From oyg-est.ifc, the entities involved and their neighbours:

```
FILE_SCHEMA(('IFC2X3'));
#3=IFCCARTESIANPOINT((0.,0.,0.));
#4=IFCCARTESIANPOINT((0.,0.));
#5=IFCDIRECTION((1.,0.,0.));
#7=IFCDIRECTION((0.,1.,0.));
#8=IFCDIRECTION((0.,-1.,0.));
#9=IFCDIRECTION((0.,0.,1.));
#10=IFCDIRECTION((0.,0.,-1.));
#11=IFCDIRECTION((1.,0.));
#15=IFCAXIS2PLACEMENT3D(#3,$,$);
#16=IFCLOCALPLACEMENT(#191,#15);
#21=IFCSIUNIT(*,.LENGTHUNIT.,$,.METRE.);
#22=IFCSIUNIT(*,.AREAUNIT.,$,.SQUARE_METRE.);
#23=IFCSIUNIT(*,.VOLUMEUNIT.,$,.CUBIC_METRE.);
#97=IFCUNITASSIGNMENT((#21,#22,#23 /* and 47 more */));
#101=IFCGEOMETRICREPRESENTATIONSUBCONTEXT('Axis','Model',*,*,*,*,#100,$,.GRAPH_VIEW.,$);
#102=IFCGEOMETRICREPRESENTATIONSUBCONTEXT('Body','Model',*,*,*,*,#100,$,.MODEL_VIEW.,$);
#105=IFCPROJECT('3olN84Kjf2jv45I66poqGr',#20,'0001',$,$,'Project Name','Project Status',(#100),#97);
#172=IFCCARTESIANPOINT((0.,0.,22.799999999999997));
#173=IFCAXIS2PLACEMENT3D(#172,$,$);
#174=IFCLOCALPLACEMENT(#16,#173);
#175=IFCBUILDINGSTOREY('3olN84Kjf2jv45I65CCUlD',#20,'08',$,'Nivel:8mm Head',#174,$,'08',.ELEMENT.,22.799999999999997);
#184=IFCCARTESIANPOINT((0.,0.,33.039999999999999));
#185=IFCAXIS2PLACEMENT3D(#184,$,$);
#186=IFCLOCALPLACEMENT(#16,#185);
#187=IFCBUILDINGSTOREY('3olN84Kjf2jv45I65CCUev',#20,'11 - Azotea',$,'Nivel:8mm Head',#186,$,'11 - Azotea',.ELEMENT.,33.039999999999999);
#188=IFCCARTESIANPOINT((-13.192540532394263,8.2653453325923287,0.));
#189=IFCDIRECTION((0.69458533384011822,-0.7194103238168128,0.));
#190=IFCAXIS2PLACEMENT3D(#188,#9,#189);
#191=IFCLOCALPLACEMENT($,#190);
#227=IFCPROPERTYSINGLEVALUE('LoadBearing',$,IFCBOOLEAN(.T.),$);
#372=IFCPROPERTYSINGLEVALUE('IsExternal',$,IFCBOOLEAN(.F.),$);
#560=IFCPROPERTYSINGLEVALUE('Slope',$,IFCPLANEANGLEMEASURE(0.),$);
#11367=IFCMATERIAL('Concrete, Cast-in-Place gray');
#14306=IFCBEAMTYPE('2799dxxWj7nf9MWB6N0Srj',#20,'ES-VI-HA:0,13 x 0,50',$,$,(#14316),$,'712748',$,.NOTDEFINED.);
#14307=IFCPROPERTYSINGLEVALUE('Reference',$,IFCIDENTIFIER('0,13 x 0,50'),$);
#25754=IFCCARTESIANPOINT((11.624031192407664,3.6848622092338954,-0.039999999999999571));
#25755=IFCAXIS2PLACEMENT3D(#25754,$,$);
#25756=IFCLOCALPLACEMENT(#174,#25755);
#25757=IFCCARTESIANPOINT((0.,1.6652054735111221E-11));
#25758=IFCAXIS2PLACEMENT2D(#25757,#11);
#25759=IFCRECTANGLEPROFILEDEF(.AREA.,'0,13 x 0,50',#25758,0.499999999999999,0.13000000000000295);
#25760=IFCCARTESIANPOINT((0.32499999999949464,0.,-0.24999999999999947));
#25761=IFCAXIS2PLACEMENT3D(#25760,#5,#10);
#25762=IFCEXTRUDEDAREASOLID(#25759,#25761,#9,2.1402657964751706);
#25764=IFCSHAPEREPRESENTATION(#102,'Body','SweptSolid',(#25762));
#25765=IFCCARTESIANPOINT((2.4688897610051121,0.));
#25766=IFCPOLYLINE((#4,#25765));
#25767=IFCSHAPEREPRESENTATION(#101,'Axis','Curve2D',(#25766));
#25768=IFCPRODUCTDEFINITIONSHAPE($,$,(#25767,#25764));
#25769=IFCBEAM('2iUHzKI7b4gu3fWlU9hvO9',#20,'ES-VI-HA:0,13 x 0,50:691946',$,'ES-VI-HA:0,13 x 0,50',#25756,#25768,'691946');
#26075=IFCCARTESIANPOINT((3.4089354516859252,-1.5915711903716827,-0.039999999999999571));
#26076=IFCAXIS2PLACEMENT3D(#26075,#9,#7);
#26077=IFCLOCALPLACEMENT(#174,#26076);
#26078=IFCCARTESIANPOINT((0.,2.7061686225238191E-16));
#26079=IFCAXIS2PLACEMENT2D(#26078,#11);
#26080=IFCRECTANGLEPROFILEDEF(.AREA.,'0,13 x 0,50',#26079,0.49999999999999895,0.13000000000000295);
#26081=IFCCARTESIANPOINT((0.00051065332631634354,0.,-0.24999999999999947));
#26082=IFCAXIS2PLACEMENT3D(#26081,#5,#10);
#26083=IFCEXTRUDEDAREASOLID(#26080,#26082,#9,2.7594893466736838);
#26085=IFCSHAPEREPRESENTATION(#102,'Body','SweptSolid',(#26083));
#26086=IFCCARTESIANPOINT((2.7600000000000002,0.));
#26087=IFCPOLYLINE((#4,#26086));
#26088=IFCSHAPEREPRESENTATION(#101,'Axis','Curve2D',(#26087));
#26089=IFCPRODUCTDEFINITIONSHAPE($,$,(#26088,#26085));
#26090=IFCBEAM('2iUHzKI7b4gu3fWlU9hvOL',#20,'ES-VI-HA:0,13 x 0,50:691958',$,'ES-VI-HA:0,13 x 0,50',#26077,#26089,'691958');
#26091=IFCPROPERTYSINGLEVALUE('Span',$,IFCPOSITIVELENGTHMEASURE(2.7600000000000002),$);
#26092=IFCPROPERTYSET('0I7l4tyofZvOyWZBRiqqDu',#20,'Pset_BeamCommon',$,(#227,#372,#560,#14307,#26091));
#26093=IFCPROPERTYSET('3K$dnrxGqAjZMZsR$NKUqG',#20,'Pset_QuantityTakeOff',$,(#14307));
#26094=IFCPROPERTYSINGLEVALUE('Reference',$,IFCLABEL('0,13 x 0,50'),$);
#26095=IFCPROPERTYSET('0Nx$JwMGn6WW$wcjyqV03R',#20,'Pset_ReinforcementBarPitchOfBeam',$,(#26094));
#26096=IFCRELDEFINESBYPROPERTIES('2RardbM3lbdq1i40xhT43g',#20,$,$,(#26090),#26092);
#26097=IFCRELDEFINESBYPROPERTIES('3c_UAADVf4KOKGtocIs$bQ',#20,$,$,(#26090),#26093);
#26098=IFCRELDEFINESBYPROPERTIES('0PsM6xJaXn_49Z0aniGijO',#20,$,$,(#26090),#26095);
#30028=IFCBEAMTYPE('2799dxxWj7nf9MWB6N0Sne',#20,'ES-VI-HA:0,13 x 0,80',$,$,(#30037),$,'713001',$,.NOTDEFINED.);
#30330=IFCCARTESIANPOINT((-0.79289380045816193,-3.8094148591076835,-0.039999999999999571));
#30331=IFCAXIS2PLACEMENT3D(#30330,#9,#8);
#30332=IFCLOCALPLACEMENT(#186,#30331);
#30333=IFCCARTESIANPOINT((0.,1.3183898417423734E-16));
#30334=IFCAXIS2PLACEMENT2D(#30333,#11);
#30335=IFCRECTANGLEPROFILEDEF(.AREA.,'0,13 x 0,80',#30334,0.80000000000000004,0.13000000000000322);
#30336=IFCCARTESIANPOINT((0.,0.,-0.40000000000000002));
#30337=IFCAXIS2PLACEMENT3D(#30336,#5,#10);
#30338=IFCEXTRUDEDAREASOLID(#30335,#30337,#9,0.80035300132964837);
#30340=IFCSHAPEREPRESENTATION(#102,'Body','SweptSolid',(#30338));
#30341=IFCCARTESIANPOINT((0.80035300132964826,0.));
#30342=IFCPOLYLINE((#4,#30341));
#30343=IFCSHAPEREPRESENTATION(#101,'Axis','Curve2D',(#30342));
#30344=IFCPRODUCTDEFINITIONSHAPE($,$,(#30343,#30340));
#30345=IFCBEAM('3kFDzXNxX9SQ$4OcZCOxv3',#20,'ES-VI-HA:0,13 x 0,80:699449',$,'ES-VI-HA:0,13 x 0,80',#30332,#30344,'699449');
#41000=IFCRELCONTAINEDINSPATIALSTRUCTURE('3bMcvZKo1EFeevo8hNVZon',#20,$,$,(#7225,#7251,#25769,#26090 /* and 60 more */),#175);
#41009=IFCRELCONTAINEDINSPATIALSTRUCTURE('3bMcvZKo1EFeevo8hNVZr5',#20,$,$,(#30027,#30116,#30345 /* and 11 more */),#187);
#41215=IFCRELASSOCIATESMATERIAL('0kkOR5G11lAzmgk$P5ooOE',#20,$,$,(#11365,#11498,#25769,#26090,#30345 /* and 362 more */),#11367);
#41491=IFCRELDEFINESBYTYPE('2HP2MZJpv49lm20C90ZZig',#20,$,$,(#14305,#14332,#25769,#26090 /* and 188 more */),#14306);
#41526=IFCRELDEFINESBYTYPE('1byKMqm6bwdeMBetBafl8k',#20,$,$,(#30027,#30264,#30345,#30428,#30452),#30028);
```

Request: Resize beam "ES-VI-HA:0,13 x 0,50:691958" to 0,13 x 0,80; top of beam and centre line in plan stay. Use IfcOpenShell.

```python
import ifcopenshell
import ifcopenshell.api.pset
import ifcopenshell.api.type
import ifcopenshell.util.element
import ifcopenshell.util.representation

model = ifcopenshell.open("oyg-est.ifc")

member = model.by_guid("2iUHzKI7b4gu3fWlU9hvOL")
source = next(p for p in model.by_type("IfcRectangleProfileDef") if p.ProfileName == "0,13 x 0,80")

body = ifcopenshell.util.representation.get_representation(member, "Model", "Body")
solid = body.Items[0]
old_profile = solid.SweptArea

# Copy the section's sizes but keep this member's own profile position.
profile = ifcopenshell.util.element.copy(model, source)
# Profiles are centred, so shift by half the change in depth to hold the top.
shift = (old_profile.XDim - profile.XDim) / 2
x, y = old_profile.Position.Location.Coordinates
up = (-1.0, 0.0)  # upwards, in the solid's own plane
location = model.createIfcCartesianPoint((x + up[0] * shift, y + up[1] * shift))
profile.Position = model.createIfcAxis2Placement2D(location, old_profile.Position.RefDirection)
solid.SweptArea = profile
if not model.get_total_inverses(old_profile):
    ifcopenshell.util.element.remove_deep2(model, old_profile)

new_type = model.by_guid("2799dxxWj7nf9MWB6N0Sne")
ifcopenshell.api.type.assign_type(
    model, related_objects=[member], relating_type=new_type, should_map_representations=False
)
member.Name = member.Name.replace("0,13 x 0,50", "0,13 x 0,80")
member.ObjectType = "ES-VI-HA:0,13 x 0,80"
pset = model.by_id(ifcopenshell.util.element.get_pset(member, "Pset_BeamCommon", should_inherit=False)["id"])
ifcopenshell.api.pset.edit_pset(model, pset=pset, properties={"Reference": "0,13 x 0,80"})
pset = model.by_id(ifcopenshell.util.element.get_pset(member, "Pset_QuantityTakeOff", should_inherit=False)["id"])
ifcopenshell.api.pset.edit_pset(model, pset=pset, properties={"Reference": "0,13 x 0,80"})
pset = model.by_id(ifcopenshell.util.element.get_pset(member, "Pset_ReinforcementBarPitchOfBeam", should_inherit=False)["id"])
ifcopenshell.api.pset.edit_pset(model, pset=pset, properties={"Reference": "0,13 x 0,80"})

print(solid.SweptArea)

model.write("oyg-est_rev.ifc")
```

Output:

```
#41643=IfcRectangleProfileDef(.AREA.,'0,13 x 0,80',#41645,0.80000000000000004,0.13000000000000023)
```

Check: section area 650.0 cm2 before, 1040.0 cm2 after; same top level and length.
